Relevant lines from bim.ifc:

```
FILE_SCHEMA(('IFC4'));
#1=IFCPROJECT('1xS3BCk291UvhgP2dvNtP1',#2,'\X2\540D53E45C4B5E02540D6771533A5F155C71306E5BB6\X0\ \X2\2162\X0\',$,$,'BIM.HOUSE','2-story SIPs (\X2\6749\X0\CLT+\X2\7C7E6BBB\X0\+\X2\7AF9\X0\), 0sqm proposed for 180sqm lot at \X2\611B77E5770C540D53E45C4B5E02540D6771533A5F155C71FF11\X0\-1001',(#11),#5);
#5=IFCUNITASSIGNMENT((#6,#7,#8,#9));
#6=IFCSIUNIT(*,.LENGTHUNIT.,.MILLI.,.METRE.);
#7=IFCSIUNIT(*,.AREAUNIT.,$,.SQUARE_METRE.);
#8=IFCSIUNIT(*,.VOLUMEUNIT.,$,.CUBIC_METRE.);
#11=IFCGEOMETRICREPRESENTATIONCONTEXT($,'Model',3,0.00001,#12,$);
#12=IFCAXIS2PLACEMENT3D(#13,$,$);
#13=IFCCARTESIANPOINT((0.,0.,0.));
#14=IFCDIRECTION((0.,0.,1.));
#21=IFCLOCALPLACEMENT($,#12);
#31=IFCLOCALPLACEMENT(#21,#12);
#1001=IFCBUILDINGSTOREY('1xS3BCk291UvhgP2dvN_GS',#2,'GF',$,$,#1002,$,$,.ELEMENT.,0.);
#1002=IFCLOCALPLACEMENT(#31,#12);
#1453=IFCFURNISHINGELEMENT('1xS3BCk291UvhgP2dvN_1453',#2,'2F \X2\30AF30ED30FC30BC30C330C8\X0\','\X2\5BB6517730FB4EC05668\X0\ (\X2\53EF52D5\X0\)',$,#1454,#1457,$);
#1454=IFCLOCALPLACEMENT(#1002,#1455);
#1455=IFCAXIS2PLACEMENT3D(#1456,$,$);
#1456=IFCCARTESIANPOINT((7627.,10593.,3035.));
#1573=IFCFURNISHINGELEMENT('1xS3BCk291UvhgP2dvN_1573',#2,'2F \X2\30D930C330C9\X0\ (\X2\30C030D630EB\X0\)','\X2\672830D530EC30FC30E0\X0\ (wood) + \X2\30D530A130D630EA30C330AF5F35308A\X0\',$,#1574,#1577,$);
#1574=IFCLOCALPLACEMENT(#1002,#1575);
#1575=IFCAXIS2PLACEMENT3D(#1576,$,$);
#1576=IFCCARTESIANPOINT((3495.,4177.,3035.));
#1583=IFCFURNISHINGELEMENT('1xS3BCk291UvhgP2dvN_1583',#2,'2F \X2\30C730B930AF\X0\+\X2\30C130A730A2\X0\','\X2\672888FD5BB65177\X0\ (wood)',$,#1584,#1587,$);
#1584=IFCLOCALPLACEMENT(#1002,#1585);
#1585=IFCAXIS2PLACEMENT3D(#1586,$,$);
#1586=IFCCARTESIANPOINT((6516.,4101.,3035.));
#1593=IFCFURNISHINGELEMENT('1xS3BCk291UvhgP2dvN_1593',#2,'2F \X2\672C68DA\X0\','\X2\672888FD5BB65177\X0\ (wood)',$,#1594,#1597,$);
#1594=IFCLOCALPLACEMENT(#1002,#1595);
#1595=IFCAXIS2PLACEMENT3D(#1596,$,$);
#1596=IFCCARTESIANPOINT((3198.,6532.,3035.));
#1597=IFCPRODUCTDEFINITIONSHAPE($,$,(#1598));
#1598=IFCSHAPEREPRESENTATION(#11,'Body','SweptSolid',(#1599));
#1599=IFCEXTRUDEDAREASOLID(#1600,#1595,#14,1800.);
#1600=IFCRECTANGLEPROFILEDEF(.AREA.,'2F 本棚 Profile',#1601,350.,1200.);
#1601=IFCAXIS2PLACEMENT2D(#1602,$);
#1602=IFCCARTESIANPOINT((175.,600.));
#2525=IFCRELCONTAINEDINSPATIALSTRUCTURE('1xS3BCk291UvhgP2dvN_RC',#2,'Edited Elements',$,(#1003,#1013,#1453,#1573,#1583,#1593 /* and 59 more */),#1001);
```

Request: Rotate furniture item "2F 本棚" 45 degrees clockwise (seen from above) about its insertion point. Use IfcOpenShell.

```python
import ifcopenshell
import ifcopenshell.api.geometry
import ifcopenshell.util.placement

model = ifcopenshell.open("bim.ifc")

item = model.by_id(1593)
matrix = ifcopenshell.util.placement.get_local_placement(item.ObjectPlacement)
matrix = matrix @ ifcopenshell.util.placement.rotation(-45, "Z")
ifcopenshell.api.geometry.edit_object_placement(model, product=item, matrix=matrix, is_si=False)

print(ifcopenshell.util.placement.get_local_placement(item.ObjectPlacement).round(3) + 0.0)

model.write("bim_rev.ifc")
```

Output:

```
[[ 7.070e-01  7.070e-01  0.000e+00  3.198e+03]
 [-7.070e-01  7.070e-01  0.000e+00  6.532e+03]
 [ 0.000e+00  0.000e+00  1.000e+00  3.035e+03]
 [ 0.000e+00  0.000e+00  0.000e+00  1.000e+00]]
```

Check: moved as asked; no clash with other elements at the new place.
